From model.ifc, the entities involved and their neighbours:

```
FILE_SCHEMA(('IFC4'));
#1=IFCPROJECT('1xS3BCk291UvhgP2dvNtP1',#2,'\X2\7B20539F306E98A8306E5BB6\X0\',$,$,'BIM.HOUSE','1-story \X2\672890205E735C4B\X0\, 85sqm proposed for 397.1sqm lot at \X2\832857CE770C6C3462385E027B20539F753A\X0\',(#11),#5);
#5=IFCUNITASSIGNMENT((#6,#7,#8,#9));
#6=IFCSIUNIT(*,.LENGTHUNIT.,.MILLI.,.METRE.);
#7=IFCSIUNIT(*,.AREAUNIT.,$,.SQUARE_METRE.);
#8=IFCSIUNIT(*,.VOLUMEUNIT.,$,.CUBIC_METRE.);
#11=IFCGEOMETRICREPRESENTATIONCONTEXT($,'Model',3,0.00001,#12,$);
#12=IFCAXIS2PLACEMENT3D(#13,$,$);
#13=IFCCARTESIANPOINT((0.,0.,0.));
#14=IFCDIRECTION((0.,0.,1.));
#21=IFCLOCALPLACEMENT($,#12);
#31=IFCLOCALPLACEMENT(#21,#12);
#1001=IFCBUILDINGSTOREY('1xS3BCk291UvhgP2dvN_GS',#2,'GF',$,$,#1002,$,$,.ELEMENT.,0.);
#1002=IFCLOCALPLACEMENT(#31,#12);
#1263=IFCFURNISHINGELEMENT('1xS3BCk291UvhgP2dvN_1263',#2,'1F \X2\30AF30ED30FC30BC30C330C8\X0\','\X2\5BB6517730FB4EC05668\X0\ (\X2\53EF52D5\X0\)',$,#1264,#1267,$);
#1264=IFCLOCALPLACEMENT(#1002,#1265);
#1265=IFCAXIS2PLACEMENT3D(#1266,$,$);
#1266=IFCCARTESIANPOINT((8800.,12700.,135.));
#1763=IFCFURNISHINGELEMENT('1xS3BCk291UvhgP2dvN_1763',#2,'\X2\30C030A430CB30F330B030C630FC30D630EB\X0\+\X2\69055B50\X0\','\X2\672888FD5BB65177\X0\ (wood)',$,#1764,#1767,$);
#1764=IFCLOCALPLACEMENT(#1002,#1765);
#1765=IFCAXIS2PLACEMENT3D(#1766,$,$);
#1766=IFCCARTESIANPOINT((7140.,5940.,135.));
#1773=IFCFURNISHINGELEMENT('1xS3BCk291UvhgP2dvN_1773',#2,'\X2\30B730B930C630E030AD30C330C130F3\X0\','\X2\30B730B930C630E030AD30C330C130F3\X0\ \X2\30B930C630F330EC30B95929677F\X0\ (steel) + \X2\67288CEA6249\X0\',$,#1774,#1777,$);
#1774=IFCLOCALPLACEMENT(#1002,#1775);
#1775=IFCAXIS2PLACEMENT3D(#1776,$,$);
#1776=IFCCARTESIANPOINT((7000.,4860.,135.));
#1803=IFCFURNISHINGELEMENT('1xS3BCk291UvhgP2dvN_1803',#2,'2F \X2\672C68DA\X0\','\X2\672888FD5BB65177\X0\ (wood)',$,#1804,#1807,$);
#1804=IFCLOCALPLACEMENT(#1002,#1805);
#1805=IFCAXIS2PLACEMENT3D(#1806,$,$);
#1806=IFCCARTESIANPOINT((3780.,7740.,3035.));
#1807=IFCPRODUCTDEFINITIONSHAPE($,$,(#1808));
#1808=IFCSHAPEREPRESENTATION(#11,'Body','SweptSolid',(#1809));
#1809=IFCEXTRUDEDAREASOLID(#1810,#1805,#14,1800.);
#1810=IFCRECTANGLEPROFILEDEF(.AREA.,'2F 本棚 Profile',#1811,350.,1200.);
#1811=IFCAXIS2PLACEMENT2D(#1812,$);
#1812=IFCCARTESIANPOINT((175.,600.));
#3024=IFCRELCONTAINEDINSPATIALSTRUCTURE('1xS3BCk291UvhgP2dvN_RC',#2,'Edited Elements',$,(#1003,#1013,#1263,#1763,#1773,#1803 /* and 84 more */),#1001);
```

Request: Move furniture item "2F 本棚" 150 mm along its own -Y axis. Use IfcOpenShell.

```python
import ifcopenshell
import ifcopenshell.api.geometry
import ifcopenshell.util.placement

model = ifcopenshell.open("model.ifc")

item = model.by_guid("1xS3BCk291UvhgP2dvN_1803")
matrix = ifcopenshell.util.placement.get_local_placement(item.ObjectPlacement)
matrix[:3, 3] -= matrix[:3, 1] * 150.0
ifcopenshell.api.geometry.edit_object_placement(model, product=item, matrix=matrix, is_si=False)

print(ifcopenshell.util.placement.get_local_placement(item.ObjectPlacement).round(3) + 0.0)

model.write("model_v2.ifc")
```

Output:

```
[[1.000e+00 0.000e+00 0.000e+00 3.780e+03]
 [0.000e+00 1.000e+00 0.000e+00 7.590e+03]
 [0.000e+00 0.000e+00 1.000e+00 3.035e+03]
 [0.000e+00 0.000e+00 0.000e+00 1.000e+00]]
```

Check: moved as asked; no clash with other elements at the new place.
